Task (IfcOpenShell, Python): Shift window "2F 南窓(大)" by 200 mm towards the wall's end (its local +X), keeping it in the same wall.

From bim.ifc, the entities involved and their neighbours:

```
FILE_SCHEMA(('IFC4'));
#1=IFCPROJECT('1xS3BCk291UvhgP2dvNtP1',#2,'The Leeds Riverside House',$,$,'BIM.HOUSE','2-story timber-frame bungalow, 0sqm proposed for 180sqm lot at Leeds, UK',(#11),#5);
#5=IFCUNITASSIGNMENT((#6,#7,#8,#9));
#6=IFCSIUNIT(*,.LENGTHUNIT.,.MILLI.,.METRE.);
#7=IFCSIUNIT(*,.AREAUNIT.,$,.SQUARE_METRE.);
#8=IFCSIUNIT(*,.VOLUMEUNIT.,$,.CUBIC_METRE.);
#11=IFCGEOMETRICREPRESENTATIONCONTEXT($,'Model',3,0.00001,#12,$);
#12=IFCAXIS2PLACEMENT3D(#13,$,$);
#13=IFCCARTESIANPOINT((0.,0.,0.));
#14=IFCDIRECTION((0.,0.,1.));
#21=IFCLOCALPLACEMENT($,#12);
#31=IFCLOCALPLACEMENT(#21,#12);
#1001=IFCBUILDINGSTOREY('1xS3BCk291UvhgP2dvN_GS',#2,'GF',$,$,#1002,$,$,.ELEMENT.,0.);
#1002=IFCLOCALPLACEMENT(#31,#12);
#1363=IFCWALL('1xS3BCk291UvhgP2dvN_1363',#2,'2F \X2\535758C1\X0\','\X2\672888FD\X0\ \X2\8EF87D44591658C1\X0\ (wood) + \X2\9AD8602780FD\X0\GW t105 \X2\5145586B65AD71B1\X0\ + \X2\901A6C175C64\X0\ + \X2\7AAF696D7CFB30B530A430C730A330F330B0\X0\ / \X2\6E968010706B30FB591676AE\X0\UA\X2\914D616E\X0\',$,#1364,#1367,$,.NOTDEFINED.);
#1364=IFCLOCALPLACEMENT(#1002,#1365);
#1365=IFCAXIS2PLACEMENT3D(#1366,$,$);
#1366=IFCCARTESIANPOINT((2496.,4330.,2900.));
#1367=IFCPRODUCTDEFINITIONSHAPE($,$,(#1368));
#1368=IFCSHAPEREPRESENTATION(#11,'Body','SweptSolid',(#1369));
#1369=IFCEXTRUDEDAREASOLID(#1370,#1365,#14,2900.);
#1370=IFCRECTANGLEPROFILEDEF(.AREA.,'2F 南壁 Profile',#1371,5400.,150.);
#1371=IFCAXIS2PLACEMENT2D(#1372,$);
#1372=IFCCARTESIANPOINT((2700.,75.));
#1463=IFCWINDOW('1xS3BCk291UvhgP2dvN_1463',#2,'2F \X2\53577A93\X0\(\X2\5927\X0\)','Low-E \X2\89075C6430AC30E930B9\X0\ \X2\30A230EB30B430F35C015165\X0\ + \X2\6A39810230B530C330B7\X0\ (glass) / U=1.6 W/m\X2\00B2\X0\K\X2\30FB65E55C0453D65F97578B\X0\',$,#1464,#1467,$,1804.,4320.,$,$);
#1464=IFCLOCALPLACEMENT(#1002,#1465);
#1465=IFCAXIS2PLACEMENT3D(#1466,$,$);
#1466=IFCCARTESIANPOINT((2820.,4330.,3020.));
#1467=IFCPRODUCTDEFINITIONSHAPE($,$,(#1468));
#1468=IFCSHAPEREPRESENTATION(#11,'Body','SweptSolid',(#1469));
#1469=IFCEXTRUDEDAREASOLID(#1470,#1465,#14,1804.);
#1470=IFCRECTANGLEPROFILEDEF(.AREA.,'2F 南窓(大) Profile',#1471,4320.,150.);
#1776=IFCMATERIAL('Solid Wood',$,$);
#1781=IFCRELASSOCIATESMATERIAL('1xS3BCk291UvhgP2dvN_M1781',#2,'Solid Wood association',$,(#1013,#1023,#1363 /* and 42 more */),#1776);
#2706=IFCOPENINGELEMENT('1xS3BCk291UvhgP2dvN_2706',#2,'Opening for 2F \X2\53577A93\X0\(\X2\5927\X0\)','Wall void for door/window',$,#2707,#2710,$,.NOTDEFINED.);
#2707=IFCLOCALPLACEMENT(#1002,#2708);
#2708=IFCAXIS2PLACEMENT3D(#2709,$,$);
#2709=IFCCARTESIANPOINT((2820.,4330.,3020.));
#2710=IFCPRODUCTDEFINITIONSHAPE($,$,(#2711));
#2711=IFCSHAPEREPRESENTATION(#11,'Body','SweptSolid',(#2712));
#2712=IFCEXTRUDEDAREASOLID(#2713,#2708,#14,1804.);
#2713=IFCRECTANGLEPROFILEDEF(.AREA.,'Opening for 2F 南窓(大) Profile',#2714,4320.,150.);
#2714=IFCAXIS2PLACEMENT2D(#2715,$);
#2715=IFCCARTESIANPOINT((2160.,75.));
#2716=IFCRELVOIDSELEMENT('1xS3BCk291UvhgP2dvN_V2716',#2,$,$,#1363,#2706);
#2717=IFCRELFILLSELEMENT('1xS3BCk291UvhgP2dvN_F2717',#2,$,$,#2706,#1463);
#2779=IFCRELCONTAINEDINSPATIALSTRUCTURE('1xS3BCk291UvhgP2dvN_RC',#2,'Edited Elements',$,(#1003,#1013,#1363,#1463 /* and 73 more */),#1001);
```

```python
import ifcopenshell
import ifcopenshell.api.geometry
import ifcopenshell.util.placement
import ifcopenshell.util.unit

model = ifcopenshell.open("bim.ifc")
unit_scale = ifcopenshell.util.unit.calculate_unit_scale(model)

window = model.by_guid("1xS3BCk291UvhgP2dvN_1463")
opening = window.FillsVoids[0].RelatingOpeningElement
wall = opening.VoidsElements[0].RelatingBuildingElement

wall_matrix = ifcopenshell.util.placement.get_local_placement(wall.ObjectPlacement)
shift = wall_matrix[:3, 0] * 0.2 / unit_scale
before = ifcopenshell.util.placement.get_local_placement(window.ObjectPlacement)[:3, 3].copy()

# The window is not placed relative to its opening, so move both.
for product in (opening, window):
    matrix = ifcopenshell.util.placement.get_local_placement(product.ObjectPlacement)
    matrix[:3, 3] += shift
    ifcopenshell.api.geometry.edit_object_placement(model, product=product, matrix=matrix, is_si=False)

after = ifcopenshell.util.placement.get_local_placement(window.ObjectPlacement)[:3, 3]
print("window moved by", (after - before).round(3) + 0.0)

model.write("bim_rev.ifc")
```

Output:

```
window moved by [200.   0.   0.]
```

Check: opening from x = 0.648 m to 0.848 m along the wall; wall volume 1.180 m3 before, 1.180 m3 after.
